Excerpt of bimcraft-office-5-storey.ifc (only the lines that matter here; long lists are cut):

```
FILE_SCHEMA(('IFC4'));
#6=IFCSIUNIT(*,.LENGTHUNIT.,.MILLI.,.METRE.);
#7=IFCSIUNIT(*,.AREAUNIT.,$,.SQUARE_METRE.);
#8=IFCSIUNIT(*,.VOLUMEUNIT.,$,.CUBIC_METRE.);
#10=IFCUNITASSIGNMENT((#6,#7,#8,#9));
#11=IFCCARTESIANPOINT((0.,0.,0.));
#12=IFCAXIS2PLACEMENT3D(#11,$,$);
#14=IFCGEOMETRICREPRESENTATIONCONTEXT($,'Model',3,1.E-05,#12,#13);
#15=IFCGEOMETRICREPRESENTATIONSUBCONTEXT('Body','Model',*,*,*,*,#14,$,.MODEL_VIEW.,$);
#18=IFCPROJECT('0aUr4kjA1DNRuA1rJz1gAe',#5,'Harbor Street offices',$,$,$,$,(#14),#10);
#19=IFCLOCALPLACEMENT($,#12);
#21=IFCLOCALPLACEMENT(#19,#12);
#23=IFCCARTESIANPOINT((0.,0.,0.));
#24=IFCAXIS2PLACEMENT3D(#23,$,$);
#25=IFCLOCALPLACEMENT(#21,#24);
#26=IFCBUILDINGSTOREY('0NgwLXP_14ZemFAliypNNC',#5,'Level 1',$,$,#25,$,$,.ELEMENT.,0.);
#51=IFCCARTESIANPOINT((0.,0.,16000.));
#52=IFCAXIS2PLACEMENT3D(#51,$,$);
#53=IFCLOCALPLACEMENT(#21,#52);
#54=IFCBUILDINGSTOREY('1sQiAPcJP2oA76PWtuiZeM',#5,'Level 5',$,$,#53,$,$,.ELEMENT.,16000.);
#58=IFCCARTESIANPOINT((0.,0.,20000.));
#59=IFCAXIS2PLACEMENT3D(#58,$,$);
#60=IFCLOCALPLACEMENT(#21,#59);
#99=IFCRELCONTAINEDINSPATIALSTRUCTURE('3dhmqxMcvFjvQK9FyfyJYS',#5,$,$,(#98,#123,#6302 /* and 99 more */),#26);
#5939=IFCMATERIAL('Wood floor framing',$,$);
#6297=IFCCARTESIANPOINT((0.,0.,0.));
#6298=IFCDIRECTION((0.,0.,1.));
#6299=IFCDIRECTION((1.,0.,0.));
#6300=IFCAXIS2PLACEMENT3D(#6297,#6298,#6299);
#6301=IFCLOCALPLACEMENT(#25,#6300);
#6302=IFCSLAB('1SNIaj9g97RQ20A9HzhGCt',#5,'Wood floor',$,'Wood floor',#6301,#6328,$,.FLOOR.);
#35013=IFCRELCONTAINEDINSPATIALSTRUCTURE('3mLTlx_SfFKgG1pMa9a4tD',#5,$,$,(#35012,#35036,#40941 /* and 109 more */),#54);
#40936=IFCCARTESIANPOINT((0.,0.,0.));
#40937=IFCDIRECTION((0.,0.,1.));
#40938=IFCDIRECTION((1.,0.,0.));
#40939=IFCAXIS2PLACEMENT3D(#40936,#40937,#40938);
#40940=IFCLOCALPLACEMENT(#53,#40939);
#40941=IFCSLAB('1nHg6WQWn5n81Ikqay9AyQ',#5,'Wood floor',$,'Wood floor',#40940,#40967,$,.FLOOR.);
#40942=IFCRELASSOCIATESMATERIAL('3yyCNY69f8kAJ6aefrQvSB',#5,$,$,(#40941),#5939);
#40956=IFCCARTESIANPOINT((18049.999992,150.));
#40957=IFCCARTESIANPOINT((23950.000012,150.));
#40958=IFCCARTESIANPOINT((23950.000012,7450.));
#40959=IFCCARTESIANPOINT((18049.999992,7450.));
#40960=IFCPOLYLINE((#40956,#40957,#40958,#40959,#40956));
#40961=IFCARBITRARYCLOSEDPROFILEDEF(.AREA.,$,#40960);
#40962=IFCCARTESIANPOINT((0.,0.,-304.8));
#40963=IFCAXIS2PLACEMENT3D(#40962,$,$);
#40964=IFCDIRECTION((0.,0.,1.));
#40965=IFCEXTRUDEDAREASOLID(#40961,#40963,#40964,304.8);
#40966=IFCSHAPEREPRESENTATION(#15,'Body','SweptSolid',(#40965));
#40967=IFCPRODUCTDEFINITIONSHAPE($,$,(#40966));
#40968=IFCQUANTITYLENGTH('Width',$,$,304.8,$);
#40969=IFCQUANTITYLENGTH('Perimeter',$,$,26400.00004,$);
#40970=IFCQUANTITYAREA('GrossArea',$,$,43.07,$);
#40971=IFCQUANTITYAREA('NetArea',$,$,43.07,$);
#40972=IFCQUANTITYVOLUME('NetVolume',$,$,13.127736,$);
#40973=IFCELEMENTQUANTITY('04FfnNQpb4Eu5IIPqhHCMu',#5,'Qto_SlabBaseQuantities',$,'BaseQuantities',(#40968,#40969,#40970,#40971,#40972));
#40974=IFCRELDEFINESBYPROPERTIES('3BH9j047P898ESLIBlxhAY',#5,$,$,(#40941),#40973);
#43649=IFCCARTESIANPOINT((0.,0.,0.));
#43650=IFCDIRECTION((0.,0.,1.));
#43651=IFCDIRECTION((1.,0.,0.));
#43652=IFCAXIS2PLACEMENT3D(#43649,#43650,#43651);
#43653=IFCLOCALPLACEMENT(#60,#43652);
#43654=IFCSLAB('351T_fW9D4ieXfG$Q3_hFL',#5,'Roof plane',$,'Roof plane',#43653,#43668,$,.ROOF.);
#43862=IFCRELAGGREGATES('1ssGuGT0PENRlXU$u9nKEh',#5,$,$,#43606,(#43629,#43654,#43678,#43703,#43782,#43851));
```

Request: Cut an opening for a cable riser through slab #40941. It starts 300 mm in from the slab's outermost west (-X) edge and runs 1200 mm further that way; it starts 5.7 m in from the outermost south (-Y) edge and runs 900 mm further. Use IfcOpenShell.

```python
import numpy as np
import ifcopenshell
import ifcopenshell.api.feature
import ifcopenshell.api.geometry
import ifcopenshell.api.pset
import ifcopenshell.api.root
import ifcopenshell.geom
import ifcopenshell.util.element
import ifcopenshell.util.placement
import ifcopenshell.util.representation
import ifcopenshell.util.shape
import ifcopenshell.util.unit

model = ifcopenshell.open("bimcraft-office-5-storey.ifc")
unit_scale = ifcopenshell.util.unit.calculate_unit_scale(model)
area_scale = ifcopenshell.util.unit.calculate_unit_scale(model, "AREAUNIT")
volume_scale = ifcopenshell.util.unit.calculate_unit_scale(model, "VOLUMEUNIT")
settings = ifcopenshell.geom.settings()


def volume(element):
    """Net volume in cubic metres, openings subtracted."""
    shape = ifcopenshell.geom.create_shape(settings, element)
    return ifcopenshell.util.shape.get_volume(shape.geometry)


slab = model.by_guid("1nHg6WQWn5n81Ikqay9AyQ")
before = volume(slab)

# Extent in the slab's own axes, in metres. The edges named are its -X and -Y sides.
slab_shape = ifcopenshell.geom.create_shape(settings, slab)
vertices = ifcopenshell.util.shape.get_vertices(slab_shape.geometry)
x_min, y_min, bottom = vertices.min(axis=0)
top = vertices[:, 2].max()

opening = ifcopenshell.api.root.create_entity(model, ifc_class="IfcOpeningElement", name="Cable riser opening", predefined_type="OPENING")
context = ifcopenshell.util.representation.get_context(model, "Model", "Body", "MODEL_VIEW")
width, depth = 1.2, 0.9
outline = [(0.0, 0.0), (width, 0.0), (width, depth), (0.0, depth), (0.0, 0.0)]
# Overshoot both faces by 50 mm so the cut is clean.
shape = ifcopenshell.api.geometry.add_slab_representation(
    model, context=context, depth=top - bottom + 0.1, polyline=outline
)
ifcopenshell.api.geometry.assign_representation(model, product=opening, representation=shape)

matrix = ifcopenshell.util.placement.get_local_placement(slab.ObjectPlacement)
matrix[:, 3] = matrix @ np.append(np.array([x_min + 0.3, y_min + 5.7, bottom - 0.05]) / unit_scale, 1.0)
ifcopenshell.api.geometry.edit_object_placement(model, product=opening, matrix=matrix, is_si=False)
ifcopenshell.api.feature.add_feature(model, feature=opening, element=slab)

after = volume(slab)

# Update the slab's stored quantities.
qto = model.by_id(ifcopenshell.util.element.get_pset(slab, "Qto_SlabBaseQuantities", should_inherit=False)["id"])
ifcopenshell.api.pset.edit_qto(model, qto=qto, properties={
    "NetArea": after / (top - bottom) / area_scale,
    "NetVolume": after / volume_scale,
})

print(f"slab volume {before:.3f} -> {after:.3f} m3")

model.write("bimcraft-office-5-storey_updated.ifc")
```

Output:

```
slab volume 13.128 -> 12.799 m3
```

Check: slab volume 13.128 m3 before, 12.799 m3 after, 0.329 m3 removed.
